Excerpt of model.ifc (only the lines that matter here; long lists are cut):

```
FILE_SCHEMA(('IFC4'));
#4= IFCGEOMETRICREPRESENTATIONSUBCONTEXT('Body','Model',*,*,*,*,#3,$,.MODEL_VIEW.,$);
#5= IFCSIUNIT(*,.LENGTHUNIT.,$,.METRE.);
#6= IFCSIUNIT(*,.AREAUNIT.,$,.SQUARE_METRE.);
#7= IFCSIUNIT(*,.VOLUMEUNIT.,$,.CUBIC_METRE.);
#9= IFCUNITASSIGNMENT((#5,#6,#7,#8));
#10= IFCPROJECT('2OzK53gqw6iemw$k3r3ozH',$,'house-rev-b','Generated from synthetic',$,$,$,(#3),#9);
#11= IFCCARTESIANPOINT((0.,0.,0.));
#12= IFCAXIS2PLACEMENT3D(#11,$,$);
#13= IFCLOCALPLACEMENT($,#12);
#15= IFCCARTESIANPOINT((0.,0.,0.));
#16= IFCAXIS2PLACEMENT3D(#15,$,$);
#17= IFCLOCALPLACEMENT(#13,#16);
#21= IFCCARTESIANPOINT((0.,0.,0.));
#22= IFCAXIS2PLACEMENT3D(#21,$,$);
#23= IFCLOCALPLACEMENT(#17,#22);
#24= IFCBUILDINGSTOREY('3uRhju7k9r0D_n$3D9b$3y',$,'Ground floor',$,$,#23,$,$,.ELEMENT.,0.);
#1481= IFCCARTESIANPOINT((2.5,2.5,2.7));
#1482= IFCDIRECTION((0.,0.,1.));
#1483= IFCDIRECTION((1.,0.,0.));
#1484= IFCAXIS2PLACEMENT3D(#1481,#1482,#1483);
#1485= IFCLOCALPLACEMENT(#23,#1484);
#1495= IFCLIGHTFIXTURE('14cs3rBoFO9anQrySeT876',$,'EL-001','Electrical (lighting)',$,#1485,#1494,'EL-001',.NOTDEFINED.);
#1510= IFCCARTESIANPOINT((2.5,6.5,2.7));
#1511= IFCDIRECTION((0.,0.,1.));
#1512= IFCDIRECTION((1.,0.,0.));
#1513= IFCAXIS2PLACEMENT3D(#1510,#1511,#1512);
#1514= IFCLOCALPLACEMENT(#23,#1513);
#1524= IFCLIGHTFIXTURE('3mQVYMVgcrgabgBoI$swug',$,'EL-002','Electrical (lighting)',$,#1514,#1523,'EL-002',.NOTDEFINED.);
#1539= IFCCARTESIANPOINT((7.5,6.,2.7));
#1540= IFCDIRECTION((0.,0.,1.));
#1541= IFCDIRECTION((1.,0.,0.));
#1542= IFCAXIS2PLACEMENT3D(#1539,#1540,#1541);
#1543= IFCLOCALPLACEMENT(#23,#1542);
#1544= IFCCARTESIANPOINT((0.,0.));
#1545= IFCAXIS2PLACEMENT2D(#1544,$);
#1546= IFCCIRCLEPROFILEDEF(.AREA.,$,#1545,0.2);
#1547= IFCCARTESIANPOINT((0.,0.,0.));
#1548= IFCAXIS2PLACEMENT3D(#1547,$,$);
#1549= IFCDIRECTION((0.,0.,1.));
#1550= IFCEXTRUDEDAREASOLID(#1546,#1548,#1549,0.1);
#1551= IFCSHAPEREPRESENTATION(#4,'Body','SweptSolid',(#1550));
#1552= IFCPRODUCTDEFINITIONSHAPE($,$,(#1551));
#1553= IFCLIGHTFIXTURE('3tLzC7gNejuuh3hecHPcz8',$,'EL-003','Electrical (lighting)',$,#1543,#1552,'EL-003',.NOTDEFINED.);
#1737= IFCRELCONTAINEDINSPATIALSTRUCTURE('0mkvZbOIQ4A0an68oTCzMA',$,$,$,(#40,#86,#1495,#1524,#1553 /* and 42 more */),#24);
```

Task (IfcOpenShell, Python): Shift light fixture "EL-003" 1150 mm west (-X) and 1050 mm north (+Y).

```python
import ifcopenshell
import ifcopenshell.api.geometry
import ifcopenshell.util.placement

model = ifcopenshell.open("model.ifc")

item = model.by_guid("3tLzC7gNejuuh3hecHPcz8")
matrix = ifcopenshell.util.placement.get_local_placement(item.ObjectPlacement)
matrix[0, 3] -= 1.15
matrix[1, 3] += 1.05
ifcopenshell.api.geometry.edit_object_placement(model, product=item, matrix=matrix, is_si=False)

print(ifcopenshell.util.placement.get_local_placement(item.ObjectPlacement).round(3) + 0.0)

model.write("model_edited.ifc")
```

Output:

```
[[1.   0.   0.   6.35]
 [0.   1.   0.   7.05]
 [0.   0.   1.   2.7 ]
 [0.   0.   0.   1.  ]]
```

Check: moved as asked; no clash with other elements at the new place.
